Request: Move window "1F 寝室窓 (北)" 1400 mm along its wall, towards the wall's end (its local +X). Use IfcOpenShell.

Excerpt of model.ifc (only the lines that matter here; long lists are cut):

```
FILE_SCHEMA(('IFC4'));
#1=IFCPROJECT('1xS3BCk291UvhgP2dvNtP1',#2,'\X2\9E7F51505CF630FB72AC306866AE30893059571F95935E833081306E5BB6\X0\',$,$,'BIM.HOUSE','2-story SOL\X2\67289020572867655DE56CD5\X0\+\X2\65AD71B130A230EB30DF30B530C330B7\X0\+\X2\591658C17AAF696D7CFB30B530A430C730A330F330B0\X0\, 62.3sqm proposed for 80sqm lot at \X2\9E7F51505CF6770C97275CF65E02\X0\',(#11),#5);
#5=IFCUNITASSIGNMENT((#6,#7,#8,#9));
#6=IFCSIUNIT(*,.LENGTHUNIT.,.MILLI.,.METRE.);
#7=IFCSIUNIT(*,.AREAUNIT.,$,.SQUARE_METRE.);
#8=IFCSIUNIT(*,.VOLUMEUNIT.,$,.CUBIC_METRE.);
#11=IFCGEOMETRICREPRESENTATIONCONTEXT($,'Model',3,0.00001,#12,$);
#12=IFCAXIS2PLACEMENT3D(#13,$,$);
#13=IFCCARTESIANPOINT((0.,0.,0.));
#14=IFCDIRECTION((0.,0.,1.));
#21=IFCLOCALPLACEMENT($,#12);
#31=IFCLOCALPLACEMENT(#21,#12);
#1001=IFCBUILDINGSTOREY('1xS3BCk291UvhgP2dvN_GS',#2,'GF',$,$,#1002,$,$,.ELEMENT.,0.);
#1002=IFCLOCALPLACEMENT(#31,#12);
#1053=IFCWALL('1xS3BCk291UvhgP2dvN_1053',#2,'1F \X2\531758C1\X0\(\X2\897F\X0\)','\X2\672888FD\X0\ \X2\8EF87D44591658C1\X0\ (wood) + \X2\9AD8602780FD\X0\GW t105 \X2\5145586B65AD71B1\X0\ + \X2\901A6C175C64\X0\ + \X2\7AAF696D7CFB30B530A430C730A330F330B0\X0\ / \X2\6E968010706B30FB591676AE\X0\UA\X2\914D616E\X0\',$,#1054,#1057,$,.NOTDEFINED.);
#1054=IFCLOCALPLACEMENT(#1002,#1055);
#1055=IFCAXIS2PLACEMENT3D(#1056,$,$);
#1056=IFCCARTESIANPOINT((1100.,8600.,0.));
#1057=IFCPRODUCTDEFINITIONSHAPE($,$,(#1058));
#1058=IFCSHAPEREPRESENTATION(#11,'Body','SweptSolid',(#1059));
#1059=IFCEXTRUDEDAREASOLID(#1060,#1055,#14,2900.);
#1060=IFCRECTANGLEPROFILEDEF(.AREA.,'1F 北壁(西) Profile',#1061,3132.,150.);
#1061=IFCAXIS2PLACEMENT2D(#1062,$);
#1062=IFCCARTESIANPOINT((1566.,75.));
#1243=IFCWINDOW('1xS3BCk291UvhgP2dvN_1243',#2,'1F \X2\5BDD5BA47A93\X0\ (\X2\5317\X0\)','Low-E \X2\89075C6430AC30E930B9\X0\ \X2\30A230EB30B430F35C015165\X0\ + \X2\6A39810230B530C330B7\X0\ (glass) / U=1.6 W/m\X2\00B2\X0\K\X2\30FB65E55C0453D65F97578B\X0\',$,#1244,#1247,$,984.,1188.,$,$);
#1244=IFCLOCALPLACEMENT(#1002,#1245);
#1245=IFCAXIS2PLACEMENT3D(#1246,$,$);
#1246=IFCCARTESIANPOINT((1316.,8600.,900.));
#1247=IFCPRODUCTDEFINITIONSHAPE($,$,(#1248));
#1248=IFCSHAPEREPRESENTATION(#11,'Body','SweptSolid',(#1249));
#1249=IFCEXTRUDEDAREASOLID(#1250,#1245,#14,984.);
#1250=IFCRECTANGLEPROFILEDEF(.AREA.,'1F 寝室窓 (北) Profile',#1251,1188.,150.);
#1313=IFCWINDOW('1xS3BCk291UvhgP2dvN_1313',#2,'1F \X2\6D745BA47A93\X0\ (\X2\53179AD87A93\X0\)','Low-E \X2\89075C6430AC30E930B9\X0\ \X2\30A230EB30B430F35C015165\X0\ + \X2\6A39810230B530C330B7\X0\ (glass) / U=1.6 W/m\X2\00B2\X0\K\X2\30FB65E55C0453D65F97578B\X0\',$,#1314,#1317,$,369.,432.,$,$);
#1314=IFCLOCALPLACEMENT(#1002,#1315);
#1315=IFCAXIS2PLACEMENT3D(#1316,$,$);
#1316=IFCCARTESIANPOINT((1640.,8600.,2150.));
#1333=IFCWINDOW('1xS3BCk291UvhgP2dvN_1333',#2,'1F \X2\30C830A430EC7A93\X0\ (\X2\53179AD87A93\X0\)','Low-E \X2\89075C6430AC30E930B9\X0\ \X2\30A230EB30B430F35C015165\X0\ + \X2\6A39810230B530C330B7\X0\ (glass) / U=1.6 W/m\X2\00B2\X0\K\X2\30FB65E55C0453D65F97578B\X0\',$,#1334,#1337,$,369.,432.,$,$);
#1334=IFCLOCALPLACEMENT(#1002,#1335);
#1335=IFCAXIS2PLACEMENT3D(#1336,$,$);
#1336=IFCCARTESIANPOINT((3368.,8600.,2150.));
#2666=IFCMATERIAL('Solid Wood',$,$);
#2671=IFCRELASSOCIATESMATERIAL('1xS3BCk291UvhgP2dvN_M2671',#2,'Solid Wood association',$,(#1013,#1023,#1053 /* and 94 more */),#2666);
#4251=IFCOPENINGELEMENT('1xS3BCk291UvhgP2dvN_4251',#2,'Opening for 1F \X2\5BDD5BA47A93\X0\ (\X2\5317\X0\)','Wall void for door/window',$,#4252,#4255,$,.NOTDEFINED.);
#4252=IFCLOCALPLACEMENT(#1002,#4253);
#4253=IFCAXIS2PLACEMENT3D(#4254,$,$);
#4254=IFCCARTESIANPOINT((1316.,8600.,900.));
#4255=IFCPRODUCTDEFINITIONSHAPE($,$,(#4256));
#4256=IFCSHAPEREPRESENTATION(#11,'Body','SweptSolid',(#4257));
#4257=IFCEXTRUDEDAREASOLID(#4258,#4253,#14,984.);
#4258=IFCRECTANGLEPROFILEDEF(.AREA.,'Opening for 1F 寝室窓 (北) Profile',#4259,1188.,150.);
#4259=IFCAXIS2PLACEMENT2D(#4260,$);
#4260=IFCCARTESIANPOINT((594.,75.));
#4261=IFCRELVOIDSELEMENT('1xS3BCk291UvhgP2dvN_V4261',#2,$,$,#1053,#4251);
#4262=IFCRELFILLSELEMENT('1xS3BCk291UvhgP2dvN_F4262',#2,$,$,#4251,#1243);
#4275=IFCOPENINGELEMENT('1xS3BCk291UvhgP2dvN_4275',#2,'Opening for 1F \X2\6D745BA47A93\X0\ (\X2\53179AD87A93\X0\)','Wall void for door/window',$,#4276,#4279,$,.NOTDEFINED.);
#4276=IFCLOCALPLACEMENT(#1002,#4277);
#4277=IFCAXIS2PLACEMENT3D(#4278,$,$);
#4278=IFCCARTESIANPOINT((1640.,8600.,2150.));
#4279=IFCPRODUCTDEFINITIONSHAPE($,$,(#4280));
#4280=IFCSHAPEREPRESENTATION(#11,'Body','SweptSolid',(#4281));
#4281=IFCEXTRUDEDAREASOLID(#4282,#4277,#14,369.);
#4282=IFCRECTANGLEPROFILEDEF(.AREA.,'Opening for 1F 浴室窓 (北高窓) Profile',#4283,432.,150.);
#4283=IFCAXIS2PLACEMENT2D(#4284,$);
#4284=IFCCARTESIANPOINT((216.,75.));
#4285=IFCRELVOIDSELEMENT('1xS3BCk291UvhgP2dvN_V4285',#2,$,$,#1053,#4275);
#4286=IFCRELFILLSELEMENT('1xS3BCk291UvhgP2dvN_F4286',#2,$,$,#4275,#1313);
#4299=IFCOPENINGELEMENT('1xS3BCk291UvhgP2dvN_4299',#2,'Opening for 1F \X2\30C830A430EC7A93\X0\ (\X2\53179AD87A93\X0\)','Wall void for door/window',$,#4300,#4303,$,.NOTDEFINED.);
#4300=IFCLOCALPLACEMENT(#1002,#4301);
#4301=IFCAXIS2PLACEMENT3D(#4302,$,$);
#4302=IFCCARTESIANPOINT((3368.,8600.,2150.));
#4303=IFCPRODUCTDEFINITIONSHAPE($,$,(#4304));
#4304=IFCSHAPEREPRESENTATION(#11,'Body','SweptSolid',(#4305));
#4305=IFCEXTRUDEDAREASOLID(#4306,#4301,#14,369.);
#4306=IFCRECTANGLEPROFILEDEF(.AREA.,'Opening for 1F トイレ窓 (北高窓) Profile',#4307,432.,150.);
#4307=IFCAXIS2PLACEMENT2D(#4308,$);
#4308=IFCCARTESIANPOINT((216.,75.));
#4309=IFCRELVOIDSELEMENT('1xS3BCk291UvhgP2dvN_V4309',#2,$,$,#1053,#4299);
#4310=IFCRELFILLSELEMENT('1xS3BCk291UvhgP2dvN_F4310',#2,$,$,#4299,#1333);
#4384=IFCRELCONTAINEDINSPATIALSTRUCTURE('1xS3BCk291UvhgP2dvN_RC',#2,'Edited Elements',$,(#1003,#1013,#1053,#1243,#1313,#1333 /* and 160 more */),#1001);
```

```python
import ifcopenshell
import ifcopenshell.api.geometry
import ifcopenshell.util.placement
import ifcopenshell.util.unit

model = ifcopenshell.open("model.ifc")
unit_scale = ifcopenshell.util.unit.calculate_unit_scale(model)

window = model.by_guid("1xS3BCk291UvhgP2dvN_1243")
opening = window.FillsVoids[0].RelatingOpeningElement
wall = opening.VoidsElements[0].RelatingBuildingElement

wall_matrix = ifcopenshell.util.placement.get_local_placement(wall.ObjectPlacement)
shift = wall_matrix[:3, 0] * 1.4 / unit_scale
before = ifcopenshell.util.placement.get_local_placement(window.ObjectPlacement)[:3, 3].copy()

# The window is not placed relative to its opening, so move both.
for product in (opening, window):
    matrix = ifcopenshell.util.placement.get_local_placement(product.ObjectPlacement)
    matrix[:3, 3] += shift
    ifcopenshell.api.geometry.edit_object_placement(model, product=product, matrix=matrix, is_si=False)

after = ifcopenshell.util.placement.get_local_placement(window.ObjectPlacement)[:3, 3]
print("window moved by", (after - before).round(3) + 0.0)

model.write("model_edited.ifc")
```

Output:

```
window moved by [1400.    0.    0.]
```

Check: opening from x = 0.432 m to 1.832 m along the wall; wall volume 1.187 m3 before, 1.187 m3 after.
